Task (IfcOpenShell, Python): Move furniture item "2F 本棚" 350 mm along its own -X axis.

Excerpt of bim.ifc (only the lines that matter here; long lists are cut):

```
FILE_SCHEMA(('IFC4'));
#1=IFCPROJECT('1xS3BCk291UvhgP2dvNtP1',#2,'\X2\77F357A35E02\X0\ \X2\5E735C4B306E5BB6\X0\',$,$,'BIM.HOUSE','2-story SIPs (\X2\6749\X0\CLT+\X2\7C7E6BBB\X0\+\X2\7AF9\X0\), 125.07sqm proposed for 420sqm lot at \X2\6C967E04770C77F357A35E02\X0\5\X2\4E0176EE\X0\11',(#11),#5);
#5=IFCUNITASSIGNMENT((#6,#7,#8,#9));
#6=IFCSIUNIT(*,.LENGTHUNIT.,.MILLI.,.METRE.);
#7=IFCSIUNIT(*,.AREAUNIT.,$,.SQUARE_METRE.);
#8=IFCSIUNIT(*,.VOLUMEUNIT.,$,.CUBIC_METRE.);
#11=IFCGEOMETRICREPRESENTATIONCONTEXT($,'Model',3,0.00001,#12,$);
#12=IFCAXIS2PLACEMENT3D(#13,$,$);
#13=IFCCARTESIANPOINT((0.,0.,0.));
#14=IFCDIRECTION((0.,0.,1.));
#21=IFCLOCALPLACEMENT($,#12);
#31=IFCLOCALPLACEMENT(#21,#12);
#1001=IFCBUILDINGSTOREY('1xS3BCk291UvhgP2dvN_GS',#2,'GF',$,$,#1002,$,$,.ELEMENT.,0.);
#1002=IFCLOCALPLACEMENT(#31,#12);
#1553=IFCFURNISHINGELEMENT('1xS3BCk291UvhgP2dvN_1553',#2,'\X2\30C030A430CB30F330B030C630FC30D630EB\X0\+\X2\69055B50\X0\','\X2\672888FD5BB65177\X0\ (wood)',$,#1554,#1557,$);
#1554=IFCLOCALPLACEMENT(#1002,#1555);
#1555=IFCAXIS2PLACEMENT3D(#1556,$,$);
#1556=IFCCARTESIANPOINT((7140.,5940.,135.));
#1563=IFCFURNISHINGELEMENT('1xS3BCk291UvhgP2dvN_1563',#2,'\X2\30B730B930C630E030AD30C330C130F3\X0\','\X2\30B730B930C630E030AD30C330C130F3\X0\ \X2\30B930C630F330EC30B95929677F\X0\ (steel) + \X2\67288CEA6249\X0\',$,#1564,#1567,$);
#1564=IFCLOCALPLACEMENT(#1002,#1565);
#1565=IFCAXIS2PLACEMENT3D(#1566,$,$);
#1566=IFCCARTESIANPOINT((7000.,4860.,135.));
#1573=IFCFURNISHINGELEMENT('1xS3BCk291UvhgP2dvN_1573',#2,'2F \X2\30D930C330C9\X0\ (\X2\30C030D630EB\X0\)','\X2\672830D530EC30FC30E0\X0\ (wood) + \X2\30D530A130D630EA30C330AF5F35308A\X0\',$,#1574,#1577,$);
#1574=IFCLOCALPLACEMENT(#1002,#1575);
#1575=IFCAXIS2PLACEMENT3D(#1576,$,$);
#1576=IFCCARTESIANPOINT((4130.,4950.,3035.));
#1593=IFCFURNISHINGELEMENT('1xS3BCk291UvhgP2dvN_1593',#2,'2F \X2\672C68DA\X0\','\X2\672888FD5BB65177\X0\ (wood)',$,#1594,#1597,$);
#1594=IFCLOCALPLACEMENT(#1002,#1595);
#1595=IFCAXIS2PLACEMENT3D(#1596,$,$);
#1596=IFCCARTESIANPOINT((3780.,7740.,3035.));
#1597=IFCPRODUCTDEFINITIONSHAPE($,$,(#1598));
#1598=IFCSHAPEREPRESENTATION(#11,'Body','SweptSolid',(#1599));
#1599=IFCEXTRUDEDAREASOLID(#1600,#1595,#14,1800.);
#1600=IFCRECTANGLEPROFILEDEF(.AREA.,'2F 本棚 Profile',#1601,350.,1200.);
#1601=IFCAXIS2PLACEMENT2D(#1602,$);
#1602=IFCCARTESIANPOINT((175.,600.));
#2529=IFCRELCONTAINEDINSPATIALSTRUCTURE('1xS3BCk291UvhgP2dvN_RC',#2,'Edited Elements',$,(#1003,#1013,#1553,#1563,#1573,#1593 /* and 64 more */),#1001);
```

```python
import ifcopenshell
import ifcopenshell.api.geometry
import ifcopenshell.util.placement
import ifcopenshell.util.unit

model = ifcopenshell.open("bim.ifc")
unit_scale = ifcopenshell.util.unit.calculate_unit_scale(model)

item = model.by_guid("1xS3BCk291UvhgP2dvN_1593")
matrix = ifcopenshell.util.placement.get_local_placement(item.ObjectPlacement)
matrix[:3, 3] -= matrix[:3, 0] * 0.35 / unit_scale
ifcopenshell.api.geometry.edit_object_placement(model, product=item, matrix=matrix, is_si=False)

print(ifcopenshell.util.placement.get_local_placement(item.ObjectPlacement).round(3) + 0.0)

model.write("bim_v2.ifc")
```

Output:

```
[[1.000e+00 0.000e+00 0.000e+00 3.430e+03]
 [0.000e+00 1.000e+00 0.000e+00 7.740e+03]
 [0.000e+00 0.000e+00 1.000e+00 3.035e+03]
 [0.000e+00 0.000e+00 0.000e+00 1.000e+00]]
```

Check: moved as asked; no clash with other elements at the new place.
